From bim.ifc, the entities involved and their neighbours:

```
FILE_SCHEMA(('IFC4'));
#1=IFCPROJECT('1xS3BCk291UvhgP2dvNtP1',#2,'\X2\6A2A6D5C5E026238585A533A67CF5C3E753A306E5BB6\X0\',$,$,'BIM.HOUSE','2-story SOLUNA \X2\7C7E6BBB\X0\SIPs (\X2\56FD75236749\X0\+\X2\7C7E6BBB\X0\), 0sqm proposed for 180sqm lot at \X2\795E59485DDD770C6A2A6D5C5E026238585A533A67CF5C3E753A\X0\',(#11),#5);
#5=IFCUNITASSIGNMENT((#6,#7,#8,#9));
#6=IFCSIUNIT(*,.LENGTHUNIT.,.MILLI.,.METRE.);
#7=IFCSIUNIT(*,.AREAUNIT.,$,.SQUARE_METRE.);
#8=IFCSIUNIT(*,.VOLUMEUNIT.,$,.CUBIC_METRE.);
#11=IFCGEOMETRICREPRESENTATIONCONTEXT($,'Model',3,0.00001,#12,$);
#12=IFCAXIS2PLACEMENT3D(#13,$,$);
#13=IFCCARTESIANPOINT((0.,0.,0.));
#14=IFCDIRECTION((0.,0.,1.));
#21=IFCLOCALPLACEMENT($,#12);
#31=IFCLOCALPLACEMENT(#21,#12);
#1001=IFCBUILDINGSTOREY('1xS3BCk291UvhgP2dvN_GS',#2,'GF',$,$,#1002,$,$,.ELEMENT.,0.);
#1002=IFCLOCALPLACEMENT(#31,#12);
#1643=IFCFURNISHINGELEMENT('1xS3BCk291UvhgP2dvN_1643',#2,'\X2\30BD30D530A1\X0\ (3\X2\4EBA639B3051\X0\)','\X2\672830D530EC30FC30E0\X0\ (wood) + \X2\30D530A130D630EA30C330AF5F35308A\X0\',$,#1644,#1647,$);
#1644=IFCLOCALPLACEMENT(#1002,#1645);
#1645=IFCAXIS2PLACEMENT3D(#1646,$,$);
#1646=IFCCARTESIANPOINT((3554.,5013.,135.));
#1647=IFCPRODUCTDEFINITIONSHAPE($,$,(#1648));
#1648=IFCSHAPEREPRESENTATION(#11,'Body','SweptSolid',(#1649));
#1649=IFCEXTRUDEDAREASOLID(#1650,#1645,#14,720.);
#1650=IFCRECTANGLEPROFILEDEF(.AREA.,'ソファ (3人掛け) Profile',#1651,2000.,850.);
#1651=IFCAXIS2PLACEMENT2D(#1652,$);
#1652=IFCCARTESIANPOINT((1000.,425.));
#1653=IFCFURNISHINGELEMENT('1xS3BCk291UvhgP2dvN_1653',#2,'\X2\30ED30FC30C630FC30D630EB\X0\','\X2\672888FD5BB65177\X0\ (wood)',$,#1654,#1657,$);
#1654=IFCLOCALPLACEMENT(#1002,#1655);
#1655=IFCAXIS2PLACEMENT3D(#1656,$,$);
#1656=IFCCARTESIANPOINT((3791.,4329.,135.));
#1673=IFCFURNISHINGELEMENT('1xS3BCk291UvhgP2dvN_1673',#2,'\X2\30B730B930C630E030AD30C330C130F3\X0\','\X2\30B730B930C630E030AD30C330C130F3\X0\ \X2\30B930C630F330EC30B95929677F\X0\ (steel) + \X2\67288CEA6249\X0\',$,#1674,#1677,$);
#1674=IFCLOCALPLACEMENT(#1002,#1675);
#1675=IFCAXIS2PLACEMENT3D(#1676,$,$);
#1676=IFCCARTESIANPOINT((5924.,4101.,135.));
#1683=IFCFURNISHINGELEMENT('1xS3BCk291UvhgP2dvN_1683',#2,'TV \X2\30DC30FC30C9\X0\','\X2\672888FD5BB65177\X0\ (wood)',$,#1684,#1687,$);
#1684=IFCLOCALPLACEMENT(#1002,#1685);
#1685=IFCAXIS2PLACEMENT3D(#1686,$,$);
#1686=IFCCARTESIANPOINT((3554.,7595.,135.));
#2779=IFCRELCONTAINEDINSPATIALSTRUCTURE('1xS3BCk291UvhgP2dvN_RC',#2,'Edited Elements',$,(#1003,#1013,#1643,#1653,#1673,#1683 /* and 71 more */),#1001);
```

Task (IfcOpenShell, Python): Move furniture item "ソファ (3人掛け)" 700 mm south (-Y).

```python
import ifcopenshell
import ifcopenshell.api.geometry
import ifcopenshell.util.placement
import ifcopenshell.util.unit

model = ifcopenshell.open("bim.ifc")
unit_scale = ifcopenshell.util.unit.calculate_unit_scale(model)

item = model.by_id(1643)
matrix = ifcopenshell.util.placement.get_local_placement(item.ObjectPlacement)
matrix[1, 3] -= 0.7 / unit_scale
ifcopenshell.api.geometry.edit_object_placement(model, product=item, matrix=matrix, is_si=False)

print(ifcopenshell.util.placement.get_local_placement(item.ObjectPlacement).round(3) + 0.0)

model.write("bim_edited.ifc")
```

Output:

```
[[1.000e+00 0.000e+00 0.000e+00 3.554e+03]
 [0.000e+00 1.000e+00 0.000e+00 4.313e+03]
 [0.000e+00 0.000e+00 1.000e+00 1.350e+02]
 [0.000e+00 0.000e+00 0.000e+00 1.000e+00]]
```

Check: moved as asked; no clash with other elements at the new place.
